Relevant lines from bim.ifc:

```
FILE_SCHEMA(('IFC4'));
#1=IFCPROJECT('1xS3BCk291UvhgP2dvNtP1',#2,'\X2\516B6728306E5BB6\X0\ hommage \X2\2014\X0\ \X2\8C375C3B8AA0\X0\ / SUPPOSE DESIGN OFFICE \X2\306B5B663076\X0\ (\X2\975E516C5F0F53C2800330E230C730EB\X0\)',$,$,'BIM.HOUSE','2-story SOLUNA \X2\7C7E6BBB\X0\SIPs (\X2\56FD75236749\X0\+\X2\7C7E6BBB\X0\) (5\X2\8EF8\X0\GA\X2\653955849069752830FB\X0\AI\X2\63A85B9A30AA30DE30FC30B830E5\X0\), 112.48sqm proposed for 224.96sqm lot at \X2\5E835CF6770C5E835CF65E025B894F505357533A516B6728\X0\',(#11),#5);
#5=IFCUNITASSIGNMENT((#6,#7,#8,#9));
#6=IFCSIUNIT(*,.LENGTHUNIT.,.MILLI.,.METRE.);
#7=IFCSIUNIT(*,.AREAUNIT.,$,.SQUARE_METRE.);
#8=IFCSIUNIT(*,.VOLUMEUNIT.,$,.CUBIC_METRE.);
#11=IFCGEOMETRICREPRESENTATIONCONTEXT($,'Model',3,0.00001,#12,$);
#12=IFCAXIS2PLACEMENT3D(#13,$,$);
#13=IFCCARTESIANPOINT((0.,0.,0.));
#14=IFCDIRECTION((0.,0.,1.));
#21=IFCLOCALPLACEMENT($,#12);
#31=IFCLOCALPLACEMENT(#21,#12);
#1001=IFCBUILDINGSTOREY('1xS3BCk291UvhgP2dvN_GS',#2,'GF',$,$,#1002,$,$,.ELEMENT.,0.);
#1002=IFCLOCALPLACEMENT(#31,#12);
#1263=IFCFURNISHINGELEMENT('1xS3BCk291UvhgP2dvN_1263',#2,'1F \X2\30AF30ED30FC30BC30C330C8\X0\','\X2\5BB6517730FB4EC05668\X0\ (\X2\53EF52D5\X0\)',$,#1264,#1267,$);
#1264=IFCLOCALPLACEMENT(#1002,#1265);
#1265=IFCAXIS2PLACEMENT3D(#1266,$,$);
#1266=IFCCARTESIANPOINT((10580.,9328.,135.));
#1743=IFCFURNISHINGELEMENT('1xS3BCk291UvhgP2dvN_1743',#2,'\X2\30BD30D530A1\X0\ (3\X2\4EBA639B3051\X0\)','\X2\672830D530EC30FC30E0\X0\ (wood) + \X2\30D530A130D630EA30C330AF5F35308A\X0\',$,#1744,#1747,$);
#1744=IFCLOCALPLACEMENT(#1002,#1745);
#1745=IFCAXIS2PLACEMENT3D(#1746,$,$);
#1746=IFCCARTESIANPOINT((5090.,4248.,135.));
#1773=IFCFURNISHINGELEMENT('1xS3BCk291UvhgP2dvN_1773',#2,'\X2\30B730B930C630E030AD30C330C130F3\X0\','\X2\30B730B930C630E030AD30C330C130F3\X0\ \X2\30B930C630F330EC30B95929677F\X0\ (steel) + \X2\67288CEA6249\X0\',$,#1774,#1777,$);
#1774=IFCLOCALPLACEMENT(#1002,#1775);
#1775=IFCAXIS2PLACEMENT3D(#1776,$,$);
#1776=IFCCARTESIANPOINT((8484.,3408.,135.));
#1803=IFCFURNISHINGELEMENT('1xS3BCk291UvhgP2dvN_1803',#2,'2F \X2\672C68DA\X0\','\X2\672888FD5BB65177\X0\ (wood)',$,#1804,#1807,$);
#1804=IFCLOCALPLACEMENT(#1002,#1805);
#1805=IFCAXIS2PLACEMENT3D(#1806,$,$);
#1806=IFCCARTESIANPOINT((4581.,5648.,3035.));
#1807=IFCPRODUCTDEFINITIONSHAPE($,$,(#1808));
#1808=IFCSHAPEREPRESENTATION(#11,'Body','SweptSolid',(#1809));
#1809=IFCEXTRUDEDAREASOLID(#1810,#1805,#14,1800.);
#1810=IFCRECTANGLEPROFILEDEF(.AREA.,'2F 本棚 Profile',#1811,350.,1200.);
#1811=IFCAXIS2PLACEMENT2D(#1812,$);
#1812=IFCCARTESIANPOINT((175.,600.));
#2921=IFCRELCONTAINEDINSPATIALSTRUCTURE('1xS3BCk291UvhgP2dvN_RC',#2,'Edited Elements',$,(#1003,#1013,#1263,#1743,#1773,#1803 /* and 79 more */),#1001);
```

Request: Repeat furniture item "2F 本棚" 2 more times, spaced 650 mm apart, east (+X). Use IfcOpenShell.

```python
import numpy as np
import ifcopenshell
import ifcopenshell.api.geometry
import ifcopenshell.api.root
import ifcopenshell.util.element
import ifcopenshell.util.placement

model = ifcopenshell.open("bim.ifc")


def reuse_history(source, copy):
    """copy_class also copies each property set's owner history, people and application; keep the originals."""
    for rel in copy.IsDefinedBy:
        if rel.is_a("IfcRelDefinesByProperties") and (history := rel.RelatingPropertyDefinition.OwnerHistory):
            rel.RelatingPropertyDefinition.OwnerHistory = source.OwnerHistory
            ifcopenshell.util.element.remove_deep2(model, history)


source = model.by_guid("1xS3BCk291UvhgP2dvN_1803")
base = ifcopenshell.util.placement.get_local_placement(source.ObjectPlacement)
step = np.array([1.0, 0.0, 0.0]) * 650.0

for i in range(1, 3):
    copy = ifcopenshell.api.root.copy_class(model, product=source)
    copy.Representation = ifcopenshell.util.element.copy_deep(
        model, source.Representation, exclude=["IfcGeometricRepresentationContext", "IfcRepresentationMap"]
    )
    reuse_history(source, copy)
    matrix = base.copy()
    matrix[:3, 3] += i * step
    print("added at", matrix[:3, 3].round(3) + 0.0)
    ifcopenshell.api.geometry.edit_object_placement(model, product=copy, matrix=matrix, is_si=False)

model.write("bim_updated.ifc")
```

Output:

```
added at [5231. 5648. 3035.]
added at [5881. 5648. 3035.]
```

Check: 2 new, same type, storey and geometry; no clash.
